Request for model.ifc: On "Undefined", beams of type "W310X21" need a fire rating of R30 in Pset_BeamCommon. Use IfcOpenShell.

First a look at what the model holds.

```python
import ifcopenshell
import ifcopenshell.util.element

model = ifcopenshell.open("model.ifc")
print(model.schema)
storey = next(s for s in model.by_type("IfcBuildingStorey") if s.Name == "Undefined")
beams = [e for e in ifcopenshell.util.element.get_decomposition(storey) if e.is_a("IfcBeam")]
seen = {}
for e in beams:
    element_type = ifcopenshell.util.element.get_type(e)
    key = (element_type.Name if element_type != e and element_type else None, ifcopenshell.util.element.get_pset(e, "Pset_BeamCommon", "FireRating"))
    seen[key] = seen.get(key, 0) + 1
for (name, value), count in sorted(seen.items(), key=str):
    print(count, "x", name, "|", value)
```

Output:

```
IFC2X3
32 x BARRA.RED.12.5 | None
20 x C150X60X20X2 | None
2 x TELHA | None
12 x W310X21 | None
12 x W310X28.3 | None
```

```python
import ifcopenshell
import ifcopenshell.api.pset
import ifcopenshell.util.element

model = ifcopenshell.open("model.ifc")

storey = next(s for s in model.by_type("IfcBuildingStorey") if s.Name == "Undefined")
beams = [e for e in ifcopenshell.util.element.get_decomposition(storey) if e.is_a("IfcBeam")]

count = 0
for e in beams:
    element_type = ifcopenshell.util.element.get_type(e)
    if element_type in (None, e) or element_type.Name != "W310X21":
        continue
    found = ifcopenshell.util.element.get_pset(e, "Pset_BeamCommon", should_inherit=False)
    if found:
        pset = model.by_id(found["id"])
        if len(ifcopenshell.util.element.get_elements_by_pset(pset)) > 1:
            pset = ifcopenshell.api.pset.unshare_pset(model, products=[e], pset=pset)[0]
    else:
        pset = ifcopenshell.api.pset.add_pset(model, product=e, name="Pset_BeamCommon")
    ifcopenshell.api.pset.edit_pset(model, pset=pset, properties={"FireRating": "R30"})
    count += 1

print(count, "beams updated")

model.write("model_rev.ifc")
```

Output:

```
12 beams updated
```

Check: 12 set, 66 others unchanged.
